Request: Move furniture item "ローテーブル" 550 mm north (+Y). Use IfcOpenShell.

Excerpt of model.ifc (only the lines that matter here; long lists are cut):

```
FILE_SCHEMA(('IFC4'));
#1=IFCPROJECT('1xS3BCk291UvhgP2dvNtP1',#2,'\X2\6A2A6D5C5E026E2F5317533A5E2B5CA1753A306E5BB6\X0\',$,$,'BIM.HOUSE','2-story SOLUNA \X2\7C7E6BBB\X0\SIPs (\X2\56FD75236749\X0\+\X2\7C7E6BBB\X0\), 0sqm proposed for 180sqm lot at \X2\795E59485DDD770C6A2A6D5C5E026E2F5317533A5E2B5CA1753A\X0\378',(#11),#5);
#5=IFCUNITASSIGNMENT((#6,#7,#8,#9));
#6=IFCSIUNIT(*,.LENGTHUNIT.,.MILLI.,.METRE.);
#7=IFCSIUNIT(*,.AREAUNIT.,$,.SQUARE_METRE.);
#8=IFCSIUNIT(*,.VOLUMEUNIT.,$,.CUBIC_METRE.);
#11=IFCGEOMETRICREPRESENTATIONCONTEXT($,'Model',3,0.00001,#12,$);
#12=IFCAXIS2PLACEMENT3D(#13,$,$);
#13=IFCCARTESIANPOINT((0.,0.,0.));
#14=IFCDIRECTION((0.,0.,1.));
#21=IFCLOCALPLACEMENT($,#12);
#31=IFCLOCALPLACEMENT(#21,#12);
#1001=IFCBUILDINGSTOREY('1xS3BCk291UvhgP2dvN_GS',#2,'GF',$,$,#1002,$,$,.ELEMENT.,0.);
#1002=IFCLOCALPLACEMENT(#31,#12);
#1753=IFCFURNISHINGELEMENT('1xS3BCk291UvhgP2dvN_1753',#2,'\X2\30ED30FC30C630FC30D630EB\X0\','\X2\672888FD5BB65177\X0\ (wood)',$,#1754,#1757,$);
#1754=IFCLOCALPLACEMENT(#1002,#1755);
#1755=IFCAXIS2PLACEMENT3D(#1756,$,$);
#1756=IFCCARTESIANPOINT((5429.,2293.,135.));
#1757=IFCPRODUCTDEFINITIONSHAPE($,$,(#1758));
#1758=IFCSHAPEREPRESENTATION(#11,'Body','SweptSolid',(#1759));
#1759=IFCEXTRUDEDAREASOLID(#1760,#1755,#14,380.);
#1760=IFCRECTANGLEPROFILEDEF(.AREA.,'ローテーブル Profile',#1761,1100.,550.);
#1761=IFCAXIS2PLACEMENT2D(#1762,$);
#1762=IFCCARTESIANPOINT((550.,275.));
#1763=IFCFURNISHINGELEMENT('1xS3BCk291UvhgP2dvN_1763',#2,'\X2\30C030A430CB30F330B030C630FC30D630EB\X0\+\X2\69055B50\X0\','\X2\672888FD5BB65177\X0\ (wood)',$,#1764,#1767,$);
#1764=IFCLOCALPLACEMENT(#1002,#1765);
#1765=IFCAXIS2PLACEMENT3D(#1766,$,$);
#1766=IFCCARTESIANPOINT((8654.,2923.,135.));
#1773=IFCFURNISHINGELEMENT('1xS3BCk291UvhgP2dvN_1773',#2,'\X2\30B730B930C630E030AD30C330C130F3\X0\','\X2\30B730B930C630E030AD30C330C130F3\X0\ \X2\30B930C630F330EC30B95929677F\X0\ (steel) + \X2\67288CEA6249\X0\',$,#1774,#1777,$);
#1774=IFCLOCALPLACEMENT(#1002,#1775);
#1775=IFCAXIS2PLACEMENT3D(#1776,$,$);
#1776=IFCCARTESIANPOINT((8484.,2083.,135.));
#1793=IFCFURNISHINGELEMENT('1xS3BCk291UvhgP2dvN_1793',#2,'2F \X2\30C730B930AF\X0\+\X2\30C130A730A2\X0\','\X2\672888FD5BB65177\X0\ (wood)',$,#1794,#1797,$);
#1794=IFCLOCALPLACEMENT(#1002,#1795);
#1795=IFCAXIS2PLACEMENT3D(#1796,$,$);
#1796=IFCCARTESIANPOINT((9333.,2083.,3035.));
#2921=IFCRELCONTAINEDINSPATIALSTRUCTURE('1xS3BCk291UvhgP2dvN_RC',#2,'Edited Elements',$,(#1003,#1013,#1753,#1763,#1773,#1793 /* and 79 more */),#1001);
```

```python
import ifcopenshell
import ifcopenshell.api.geometry
import ifcopenshell.util.placement

model = ifcopenshell.open("model.ifc")

item = model.by_guid("1xS3BCk291UvhgP2dvN_1753")
matrix = ifcopenshell.util.placement.get_local_placement(item.ObjectPlacement)
matrix[1, 3] += 550.0
ifcopenshell.api.geometry.edit_object_placement(model, product=item, matrix=matrix, is_si=False)

print(ifcopenshell.util.placement.get_local_placement(item.ObjectPlacement).round(3) + 0.0)

model.write("model_edited.ifc")
```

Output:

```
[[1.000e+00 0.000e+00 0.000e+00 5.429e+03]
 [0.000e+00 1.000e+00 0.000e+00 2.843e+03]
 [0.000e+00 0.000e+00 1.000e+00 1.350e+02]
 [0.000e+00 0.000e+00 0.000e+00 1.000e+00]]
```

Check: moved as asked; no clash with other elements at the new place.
